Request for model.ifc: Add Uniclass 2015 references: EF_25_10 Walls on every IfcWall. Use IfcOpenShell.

First a look at what the model holds.

```python
import ifcopenshell

model = ifcopenshell.open("model.ifc")
print(model.schema)
print("classifications:", [c.Name for c in model.by_type("IfcClassification")])
for ifc_class in ("IfcDoor", "IfcRoof", "IfcStair", "IfcWall", "IfcWindow"):
    print(ifc_class, len(model.by_type(ifc_class)))
```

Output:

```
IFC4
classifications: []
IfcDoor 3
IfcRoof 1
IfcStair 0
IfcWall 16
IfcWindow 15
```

```python
import ifcopenshell
import ifcopenshell.api.classification

model = ifcopenshell.open("model.ifc")

system = ifcopenshell.api.classification.add_classification(model, classification="Uniclass 2015")

codes = {
    "IfcWall": ("EF_25_10", "Walls"),
}
for ifc_class, (code, name) in codes.items():
    products = model.by_type(ifc_class)
    ifcopenshell.api.classification.add_reference(
        model, products=products, classification=system, identification=code, name=name
    )
    print(code, len(products))

model.write("model_v2.ifc")
```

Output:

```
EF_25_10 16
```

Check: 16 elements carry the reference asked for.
